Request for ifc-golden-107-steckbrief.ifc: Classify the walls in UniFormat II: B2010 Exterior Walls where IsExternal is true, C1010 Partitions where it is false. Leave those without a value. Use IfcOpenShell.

First a look at what the model holds.

```python
import ifcopenshell
import ifcopenshell.util.element

model = ifcopenshell.open("ifc-golden-107-steckbrief.ifc")
print(model.schema)
print("classifications:", [c.Name for c in model.by_type("IfcClassification")])
values = [ifcopenshell.util.element.get_pset(e, "Pset_WallCommon", "IsExternal") for e in model.by_type("IfcWall")]
for value in (True, False, None):
    print("IsExternal", value, values.count(value))
```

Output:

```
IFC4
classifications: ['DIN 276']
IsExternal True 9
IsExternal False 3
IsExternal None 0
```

```python
import ifcopenshell
import ifcopenshell.api.classification
import ifcopenshell.util.element

model = ifcopenshell.open("ifc-golden-107-steckbrief.ifc")

system = ifcopenshell.api.classification.add_classification(model, classification="UniFormat II")

walls = model.by_type("IfcWall")
external = {e: ifcopenshell.util.element.get_pset(e, "Pset_WallCommon", "IsExternal") for e in walls}
for flag, code, name in ((True, "B2010", "Exterior Walls"), (False, "C1010", "Partitions")):
    products = [e for e in walls if external[e] is flag]
    ifcopenshell.api.classification.add_reference(
        model, products=products, classification=system, identification=code, name=name
    )
    print(code, len(products))

model.write("ifc-golden-107-steckbrief_updated.ifc")
```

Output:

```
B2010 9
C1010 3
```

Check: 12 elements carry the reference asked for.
